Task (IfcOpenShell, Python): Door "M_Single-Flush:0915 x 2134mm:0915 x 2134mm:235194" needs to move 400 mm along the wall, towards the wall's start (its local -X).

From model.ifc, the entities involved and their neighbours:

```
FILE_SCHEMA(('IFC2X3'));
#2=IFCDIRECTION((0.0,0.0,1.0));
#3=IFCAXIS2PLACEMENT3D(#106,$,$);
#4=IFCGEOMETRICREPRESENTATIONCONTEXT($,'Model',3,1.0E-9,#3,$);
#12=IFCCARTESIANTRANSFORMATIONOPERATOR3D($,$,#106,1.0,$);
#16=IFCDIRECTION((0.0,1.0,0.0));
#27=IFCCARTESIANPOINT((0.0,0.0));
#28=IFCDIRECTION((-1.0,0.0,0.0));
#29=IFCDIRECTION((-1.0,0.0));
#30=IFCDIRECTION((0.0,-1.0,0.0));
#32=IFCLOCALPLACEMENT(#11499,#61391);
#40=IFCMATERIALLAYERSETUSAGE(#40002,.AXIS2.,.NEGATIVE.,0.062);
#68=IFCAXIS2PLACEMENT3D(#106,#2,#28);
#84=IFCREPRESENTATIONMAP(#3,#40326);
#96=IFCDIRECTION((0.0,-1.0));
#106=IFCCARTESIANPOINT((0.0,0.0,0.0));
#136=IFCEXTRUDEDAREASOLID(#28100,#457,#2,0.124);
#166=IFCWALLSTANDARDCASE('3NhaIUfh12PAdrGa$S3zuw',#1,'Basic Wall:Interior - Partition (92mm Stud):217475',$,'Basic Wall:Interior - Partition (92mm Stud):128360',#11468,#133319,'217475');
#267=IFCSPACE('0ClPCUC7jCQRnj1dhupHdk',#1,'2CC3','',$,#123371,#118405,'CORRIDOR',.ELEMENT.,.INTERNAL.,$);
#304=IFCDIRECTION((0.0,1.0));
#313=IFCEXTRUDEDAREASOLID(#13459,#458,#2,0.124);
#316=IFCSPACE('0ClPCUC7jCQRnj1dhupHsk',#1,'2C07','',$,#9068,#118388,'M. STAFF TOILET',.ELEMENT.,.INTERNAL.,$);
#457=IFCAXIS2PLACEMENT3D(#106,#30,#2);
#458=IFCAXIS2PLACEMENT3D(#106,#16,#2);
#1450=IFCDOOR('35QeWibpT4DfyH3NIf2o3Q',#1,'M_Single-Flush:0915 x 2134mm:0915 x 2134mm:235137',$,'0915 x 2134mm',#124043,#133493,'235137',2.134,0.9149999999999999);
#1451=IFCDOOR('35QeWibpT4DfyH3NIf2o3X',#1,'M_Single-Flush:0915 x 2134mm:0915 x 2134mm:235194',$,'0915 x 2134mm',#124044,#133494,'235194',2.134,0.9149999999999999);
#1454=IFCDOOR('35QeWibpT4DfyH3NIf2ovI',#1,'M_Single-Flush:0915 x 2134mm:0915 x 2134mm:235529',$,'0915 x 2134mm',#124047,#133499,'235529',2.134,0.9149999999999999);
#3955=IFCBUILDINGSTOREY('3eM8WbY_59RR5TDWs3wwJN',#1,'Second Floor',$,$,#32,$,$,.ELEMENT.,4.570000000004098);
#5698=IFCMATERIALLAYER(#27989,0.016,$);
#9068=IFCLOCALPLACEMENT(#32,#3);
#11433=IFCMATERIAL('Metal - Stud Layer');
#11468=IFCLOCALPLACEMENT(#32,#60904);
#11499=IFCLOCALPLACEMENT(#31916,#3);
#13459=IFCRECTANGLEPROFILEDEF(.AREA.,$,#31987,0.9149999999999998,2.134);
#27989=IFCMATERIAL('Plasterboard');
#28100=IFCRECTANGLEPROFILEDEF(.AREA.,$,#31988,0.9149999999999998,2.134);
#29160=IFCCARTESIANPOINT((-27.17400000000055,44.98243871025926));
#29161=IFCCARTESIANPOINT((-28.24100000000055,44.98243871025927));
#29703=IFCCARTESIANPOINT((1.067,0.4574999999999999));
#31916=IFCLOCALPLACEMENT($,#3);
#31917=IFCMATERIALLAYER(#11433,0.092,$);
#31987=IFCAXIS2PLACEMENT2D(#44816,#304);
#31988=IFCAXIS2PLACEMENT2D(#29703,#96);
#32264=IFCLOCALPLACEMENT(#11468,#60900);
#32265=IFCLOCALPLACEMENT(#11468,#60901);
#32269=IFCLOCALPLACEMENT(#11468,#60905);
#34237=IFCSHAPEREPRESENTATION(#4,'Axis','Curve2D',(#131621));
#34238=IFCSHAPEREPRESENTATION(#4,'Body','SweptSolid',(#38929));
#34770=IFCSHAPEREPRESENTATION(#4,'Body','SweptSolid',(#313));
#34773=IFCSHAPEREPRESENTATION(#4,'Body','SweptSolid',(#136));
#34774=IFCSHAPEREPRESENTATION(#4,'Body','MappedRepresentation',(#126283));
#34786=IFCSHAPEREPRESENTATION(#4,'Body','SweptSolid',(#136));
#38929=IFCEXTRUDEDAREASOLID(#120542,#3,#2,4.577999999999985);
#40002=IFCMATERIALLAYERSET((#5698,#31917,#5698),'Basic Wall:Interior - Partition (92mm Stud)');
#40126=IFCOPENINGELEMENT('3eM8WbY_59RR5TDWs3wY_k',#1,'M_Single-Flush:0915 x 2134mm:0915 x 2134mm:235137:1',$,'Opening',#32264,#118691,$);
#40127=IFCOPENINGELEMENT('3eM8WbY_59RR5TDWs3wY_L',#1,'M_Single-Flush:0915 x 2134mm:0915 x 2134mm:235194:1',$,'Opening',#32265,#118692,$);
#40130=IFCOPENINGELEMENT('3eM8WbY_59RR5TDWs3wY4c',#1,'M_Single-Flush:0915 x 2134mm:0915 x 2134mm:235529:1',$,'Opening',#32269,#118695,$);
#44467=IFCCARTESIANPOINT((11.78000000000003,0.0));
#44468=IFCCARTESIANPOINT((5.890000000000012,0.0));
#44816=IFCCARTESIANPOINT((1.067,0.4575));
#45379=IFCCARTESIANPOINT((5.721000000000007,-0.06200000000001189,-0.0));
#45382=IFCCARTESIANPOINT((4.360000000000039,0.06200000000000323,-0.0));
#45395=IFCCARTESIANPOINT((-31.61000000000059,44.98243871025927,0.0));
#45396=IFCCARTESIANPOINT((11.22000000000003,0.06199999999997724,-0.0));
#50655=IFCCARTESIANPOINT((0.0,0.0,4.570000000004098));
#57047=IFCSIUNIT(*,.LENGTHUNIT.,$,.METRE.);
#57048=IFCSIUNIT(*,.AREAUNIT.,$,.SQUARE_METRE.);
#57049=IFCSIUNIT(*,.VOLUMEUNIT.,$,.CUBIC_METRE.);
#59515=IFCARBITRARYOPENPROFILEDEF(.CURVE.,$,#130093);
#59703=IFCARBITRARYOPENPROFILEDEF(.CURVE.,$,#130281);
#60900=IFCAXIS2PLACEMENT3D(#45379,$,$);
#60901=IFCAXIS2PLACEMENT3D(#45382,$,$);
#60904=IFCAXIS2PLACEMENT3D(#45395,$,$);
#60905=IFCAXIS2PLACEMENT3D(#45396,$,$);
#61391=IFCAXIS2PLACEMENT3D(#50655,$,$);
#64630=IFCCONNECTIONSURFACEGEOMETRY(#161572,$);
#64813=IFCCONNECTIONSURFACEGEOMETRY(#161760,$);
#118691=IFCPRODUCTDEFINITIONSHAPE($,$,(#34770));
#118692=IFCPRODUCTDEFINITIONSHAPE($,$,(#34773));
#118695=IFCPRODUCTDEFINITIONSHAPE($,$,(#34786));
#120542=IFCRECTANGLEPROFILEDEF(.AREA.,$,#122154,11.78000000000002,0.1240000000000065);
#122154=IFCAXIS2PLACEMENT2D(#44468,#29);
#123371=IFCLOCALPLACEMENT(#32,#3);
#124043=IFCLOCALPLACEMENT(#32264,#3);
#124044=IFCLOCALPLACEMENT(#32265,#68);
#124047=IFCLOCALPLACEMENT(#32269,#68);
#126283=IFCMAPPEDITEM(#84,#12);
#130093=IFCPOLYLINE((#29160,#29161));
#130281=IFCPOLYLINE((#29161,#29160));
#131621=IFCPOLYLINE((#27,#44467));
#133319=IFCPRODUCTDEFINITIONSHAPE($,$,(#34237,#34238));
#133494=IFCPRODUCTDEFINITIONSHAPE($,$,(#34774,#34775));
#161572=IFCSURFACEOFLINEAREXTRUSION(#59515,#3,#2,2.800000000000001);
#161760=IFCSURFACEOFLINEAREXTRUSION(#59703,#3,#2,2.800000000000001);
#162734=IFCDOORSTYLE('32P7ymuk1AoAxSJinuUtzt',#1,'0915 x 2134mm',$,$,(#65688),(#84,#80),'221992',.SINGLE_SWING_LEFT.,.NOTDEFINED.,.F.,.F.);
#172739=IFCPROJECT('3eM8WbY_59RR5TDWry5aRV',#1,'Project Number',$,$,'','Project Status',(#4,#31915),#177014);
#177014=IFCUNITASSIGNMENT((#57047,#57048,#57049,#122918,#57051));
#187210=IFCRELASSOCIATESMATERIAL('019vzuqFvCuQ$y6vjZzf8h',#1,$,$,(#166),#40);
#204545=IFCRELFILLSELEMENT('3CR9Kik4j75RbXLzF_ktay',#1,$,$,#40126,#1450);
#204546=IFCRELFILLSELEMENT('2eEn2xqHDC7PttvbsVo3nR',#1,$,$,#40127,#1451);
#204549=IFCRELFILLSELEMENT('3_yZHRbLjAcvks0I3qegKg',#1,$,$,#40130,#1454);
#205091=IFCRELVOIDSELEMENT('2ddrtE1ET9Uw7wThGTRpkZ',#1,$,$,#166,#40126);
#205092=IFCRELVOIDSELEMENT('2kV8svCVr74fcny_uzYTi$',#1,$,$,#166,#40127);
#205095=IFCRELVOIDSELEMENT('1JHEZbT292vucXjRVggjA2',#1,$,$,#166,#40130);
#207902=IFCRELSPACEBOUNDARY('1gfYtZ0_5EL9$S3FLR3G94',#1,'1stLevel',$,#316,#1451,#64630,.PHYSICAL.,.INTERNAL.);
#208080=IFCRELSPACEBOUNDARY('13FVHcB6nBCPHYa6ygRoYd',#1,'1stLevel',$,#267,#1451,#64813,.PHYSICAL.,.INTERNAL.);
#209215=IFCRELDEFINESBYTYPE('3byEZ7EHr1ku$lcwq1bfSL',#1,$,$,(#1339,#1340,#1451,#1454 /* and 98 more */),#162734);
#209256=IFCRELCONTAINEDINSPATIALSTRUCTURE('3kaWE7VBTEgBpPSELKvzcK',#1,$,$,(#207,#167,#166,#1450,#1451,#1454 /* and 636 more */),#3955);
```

```python
import numpy as np
import ifcopenshell
import ifcopenshell.api.geometry
import ifcopenshell.util.placement
import ifcopenshell.util.unit

model = ifcopenshell.open("model.ifc")
unit_scale = ifcopenshell.util.unit.calculate_unit_scale(model)

door = model.by_guid("35QeWibpT4DfyH3NIf2o3X")
opening = door.FillsVoids[0].RelatingOpeningElement
wall = opening.VoidsElements[0].RelatingBuildingElement

wall_matrix = ifcopenshell.util.placement.get_local_placement(wall.ObjectPlacement)
shift = wall_matrix[:3, 0] * -0.4 / unit_scale
before = ifcopenshell.util.placement.get_local_placement(door.ObjectPlacement)[:3, 3].copy()

# The door is placed relative to its opening, so it follows when the opening moves.
matrix = ifcopenshell.util.placement.get_local_placement(opening.ObjectPlacement)
matrix[:3, 3] += shift
ifcopenshell.api.geometry.edit_object_placement(
    model, product=opening, matrix=matrix, is_si=False, should_transform_children=True
)

# Space boundary surfaces are stored in each space's coordinates; move them too.
for rel in door.ProvidesBoundaries:
    if not rel.ConnectionGeometry:
        continue
    surface = rel.ConnectionGeometry.SurfaceOnRelatingElement
    space_matrix = ifcopenshell.util.placement.get_local_placement(rel.RelatingSpace.ObjectPlacement)
    point = np.array(surface.Position.Location.Coordinates) + space_matrix[:3, :3].T @ shift
    surface.Position = model.createIfcAxis2Placement3D(
        model.createIfcCartesianPoint(point.tolist()), surface.Position.Axis, surface.Position.RefDirection
    )

after = ifcopenshell.util.placement.get_local_placement(door.ObjectPlacement)[:3, 3]
print("door moved by", (after - before).round(3) + 0.0)

model.write("model-out.ifc")
```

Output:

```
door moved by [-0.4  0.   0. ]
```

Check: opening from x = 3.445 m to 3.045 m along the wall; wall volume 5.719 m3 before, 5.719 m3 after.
